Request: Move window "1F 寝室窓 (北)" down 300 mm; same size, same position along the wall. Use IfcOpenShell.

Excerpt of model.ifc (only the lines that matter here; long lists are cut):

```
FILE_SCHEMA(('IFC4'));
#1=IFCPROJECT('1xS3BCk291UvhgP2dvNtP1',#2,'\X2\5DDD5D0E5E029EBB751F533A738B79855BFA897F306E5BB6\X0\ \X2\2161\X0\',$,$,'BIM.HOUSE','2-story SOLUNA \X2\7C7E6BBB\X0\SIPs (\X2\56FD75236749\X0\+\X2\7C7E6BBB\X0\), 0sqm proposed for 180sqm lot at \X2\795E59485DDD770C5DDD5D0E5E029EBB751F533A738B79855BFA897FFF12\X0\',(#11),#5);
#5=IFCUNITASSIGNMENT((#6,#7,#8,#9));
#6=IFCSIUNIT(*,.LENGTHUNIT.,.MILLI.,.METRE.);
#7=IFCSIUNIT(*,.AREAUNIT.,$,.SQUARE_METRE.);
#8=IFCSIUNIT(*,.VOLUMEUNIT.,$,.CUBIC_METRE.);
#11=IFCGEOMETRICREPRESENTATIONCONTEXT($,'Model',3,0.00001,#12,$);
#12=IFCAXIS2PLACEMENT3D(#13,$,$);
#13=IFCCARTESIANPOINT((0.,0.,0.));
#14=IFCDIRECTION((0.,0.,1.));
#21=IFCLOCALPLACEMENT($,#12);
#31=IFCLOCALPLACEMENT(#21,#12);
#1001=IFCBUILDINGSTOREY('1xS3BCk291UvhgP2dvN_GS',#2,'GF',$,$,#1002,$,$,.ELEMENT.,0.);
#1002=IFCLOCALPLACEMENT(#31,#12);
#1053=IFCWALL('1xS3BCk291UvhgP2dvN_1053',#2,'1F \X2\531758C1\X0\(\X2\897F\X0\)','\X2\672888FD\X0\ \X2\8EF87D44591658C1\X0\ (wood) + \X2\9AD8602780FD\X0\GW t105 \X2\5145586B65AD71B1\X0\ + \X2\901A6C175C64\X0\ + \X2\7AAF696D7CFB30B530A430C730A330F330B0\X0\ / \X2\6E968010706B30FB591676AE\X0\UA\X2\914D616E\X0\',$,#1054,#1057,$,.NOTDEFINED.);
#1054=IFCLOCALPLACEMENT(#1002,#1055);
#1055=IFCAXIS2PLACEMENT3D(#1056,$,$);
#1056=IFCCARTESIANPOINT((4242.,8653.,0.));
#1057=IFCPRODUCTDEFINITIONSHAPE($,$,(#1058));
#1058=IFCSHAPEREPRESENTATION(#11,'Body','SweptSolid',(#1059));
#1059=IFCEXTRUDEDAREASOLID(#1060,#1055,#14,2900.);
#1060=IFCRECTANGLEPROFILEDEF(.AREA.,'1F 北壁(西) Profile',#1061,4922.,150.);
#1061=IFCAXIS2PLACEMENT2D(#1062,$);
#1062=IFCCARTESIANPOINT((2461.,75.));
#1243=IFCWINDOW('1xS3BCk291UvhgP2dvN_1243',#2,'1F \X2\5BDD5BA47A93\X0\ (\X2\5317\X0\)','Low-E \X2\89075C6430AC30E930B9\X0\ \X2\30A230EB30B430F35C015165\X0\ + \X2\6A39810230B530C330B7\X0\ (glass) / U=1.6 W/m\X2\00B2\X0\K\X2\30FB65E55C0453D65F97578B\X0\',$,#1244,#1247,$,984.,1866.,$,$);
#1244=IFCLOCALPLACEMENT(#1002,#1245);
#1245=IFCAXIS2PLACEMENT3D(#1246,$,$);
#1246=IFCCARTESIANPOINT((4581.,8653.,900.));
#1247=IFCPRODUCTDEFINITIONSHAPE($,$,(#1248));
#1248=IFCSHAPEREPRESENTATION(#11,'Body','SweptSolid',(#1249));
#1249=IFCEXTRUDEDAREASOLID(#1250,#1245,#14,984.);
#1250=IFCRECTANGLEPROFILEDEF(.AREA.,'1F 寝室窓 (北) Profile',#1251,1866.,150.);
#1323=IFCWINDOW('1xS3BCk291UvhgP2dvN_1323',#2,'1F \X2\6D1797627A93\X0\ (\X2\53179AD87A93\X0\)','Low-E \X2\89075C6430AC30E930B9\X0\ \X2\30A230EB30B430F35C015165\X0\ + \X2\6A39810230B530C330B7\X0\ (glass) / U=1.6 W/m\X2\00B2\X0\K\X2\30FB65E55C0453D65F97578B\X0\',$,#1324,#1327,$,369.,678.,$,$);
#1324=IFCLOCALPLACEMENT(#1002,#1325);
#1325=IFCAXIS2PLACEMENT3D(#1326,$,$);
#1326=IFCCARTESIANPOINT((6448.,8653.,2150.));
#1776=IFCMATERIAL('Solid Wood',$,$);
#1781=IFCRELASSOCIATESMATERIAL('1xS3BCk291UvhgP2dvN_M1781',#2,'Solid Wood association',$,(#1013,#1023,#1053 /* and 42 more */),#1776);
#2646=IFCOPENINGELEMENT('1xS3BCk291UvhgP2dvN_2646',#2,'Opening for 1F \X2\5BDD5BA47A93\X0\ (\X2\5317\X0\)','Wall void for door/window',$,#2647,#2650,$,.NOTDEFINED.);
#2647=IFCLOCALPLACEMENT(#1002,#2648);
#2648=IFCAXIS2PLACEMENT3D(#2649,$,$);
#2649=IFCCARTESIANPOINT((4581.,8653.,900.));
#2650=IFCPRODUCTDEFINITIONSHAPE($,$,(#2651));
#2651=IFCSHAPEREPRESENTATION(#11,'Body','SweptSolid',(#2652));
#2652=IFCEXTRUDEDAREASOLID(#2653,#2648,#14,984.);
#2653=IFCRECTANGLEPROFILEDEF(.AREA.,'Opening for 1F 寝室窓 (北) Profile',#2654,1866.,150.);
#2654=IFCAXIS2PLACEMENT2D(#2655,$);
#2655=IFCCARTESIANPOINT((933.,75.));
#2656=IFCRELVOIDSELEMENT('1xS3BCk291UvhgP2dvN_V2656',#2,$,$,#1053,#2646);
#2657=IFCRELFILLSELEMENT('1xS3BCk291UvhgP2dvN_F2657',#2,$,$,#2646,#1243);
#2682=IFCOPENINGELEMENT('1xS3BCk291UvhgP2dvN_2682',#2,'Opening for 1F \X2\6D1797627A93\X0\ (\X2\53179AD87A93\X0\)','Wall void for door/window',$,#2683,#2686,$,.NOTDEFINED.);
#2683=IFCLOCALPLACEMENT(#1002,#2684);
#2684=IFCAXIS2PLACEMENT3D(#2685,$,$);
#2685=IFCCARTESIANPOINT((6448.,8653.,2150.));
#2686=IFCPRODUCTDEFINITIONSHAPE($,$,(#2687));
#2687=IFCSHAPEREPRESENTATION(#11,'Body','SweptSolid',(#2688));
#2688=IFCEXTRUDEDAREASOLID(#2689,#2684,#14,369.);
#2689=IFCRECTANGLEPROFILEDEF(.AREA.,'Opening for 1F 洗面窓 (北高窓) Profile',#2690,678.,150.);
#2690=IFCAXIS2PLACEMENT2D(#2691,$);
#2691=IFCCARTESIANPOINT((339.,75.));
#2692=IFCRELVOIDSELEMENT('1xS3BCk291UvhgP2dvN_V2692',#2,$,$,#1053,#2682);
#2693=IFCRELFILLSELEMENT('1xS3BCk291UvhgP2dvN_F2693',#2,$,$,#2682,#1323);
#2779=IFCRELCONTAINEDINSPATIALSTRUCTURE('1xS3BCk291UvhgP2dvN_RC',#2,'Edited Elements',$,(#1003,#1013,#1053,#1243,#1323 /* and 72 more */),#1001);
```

```python
import numpy as np
import ifcopenshell
import ifcopenshell.api.geometry
import ifcopenshell.util.placement
import ifcopenshell.util.unit

model = ifcopenshell.open("model.ifc")
unit_scale = ifcopenshell.util.unit.calculate_unit_scale(model)

window = model.by_guid("1xS3BCk291UvhgP2dvN_1243")
opening = window.FillsVoids[0].RelatingOpeningElement
dz = -0.3 / unit_scale

shift = np.array([0.0, 0.0, dz])
# The window is not placed relative to its opening, so move both.
for product in (opening, window):
    matrix = ifcopenshell.util.placement.get_local_placement(product.ObjectPlacement)
    matrix[:3, 3] += shift
    ifcopenshell.api.geometry.edit_object_placement(model, product=product, matrix=matrix, is_si=False)

print(f"moved by {dz * unit_scale:+.3f} m")

model.write("model_rev.ifc")
```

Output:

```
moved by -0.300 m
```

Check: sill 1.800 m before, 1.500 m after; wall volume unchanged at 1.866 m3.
